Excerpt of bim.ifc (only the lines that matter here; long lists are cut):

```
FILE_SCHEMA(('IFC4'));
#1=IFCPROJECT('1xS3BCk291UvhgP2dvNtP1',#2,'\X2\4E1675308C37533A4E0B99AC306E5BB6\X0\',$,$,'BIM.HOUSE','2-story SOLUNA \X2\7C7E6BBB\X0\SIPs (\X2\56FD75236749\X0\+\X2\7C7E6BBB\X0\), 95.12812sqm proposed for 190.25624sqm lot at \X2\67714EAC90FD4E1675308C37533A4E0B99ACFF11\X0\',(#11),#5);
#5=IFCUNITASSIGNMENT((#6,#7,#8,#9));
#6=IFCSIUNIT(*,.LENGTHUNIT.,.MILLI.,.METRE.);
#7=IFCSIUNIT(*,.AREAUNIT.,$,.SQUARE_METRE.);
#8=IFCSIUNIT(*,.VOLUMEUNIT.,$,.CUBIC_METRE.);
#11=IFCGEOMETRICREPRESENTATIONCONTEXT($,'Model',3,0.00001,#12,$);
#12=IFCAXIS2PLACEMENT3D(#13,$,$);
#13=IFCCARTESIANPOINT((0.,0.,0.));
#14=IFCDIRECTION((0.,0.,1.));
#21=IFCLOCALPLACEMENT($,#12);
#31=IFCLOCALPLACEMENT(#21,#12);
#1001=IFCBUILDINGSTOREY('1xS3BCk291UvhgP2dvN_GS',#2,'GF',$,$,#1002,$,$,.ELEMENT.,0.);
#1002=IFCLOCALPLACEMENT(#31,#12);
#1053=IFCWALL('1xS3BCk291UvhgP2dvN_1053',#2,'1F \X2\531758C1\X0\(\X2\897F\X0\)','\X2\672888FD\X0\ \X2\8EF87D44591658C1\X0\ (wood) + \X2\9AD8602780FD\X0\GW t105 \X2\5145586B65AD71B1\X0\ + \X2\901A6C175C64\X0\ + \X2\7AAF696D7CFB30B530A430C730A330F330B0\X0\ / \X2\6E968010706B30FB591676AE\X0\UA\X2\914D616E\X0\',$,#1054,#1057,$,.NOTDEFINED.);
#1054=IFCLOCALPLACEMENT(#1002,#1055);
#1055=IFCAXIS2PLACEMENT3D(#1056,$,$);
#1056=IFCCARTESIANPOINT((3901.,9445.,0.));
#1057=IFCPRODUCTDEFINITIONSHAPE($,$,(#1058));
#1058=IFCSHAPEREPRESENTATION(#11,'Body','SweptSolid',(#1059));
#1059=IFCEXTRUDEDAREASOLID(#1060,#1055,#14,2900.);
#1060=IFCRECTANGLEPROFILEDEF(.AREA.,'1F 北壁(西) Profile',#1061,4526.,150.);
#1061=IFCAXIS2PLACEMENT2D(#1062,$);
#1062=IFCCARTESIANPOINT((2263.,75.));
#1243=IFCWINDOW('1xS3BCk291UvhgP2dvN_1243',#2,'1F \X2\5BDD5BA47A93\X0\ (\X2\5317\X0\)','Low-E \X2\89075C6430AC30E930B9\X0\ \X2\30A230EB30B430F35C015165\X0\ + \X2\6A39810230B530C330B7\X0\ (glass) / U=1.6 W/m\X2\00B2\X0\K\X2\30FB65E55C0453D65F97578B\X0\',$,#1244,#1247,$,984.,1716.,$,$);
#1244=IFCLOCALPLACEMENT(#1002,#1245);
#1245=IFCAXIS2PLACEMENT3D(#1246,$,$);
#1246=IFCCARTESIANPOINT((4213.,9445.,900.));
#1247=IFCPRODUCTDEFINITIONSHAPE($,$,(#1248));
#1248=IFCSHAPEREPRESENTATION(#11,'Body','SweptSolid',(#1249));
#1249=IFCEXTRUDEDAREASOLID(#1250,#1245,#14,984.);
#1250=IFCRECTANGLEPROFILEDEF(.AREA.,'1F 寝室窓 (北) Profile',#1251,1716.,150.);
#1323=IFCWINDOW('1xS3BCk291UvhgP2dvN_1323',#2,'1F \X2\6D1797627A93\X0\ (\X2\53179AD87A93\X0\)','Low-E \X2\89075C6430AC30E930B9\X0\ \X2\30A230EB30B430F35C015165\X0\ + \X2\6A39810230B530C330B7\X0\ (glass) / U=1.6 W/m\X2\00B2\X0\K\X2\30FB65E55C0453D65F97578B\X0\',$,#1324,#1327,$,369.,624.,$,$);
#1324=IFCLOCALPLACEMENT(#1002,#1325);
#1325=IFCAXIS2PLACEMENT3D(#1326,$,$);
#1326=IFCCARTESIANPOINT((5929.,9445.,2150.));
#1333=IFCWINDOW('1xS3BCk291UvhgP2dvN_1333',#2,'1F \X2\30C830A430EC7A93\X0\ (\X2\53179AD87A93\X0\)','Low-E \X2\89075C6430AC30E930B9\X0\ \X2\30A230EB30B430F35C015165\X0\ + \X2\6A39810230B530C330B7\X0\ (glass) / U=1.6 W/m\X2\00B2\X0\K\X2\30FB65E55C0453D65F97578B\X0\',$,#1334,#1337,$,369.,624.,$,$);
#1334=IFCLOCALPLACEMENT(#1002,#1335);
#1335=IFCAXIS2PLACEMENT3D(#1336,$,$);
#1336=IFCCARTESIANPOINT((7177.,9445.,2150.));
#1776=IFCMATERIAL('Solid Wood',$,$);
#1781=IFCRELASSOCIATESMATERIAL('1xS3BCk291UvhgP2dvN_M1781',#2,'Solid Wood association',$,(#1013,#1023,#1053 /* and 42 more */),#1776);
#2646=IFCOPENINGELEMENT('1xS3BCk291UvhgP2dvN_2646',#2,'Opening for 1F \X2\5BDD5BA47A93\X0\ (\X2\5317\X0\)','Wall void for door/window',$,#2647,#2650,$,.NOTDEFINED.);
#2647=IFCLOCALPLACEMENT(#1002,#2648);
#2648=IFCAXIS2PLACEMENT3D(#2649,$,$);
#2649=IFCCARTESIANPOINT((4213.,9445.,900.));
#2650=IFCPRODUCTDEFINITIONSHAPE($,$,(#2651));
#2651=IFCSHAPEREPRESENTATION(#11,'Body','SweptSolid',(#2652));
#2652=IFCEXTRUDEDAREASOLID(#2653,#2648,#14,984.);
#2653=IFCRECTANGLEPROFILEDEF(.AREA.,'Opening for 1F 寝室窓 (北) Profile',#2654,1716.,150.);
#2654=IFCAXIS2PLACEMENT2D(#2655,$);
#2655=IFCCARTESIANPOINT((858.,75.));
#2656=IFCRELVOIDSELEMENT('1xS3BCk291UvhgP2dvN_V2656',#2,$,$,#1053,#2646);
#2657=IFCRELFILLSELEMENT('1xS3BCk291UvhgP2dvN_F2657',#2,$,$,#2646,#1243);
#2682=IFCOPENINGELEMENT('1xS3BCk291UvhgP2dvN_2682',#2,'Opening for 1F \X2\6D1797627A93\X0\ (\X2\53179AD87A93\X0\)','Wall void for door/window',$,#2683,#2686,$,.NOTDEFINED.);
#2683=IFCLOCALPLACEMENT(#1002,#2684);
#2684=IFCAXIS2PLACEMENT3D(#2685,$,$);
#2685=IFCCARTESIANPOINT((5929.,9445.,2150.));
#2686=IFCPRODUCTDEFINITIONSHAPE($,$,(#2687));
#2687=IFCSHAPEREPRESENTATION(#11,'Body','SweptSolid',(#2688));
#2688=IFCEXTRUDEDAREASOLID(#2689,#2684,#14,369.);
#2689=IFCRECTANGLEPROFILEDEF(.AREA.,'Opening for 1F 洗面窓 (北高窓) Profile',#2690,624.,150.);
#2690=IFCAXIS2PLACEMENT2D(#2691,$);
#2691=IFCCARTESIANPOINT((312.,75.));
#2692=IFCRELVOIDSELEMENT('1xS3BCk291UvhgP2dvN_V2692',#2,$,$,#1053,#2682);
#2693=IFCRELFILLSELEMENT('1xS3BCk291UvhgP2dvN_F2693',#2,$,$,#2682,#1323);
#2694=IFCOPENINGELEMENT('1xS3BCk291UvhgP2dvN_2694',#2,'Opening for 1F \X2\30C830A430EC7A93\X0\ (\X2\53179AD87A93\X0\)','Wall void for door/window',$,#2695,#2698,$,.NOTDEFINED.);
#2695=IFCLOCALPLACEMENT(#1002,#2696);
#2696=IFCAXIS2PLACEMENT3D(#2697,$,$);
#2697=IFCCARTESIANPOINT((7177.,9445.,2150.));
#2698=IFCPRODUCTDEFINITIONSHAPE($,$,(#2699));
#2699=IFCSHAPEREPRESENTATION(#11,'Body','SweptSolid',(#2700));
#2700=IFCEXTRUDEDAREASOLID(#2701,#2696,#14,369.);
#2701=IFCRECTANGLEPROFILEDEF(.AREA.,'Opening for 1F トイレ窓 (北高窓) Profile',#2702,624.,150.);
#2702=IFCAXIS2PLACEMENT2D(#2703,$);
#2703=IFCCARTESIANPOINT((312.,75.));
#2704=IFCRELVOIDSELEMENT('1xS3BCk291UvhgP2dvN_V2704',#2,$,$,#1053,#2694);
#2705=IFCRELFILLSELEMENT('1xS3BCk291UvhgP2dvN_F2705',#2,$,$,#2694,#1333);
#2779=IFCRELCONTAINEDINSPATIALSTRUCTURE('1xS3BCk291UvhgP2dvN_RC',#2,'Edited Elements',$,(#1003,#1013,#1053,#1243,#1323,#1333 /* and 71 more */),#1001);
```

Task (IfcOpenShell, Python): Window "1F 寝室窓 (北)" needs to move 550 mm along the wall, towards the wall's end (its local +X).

```python
import ifcopenshell
import ifcopenshell.api.geometry
import ifcopenshell.util.placement
import ifcopenshell.util.unit

model = ifcopenshell.open("bim.ifc")
unit_scale = ifcopenshell.util.unit.calculate_unit_scale(model)

window = model.by_guid("1xS3BCk291UvhgP2dvN_1243")
opening = window.FillsVoids[0].RelatingOpeningElement
wall = opening.VoidsElements[0].RelatingBuildingElement

wall_matrix = ifcopenshell.util.placement.get_local_placement(wall.ObjectPlacement)
shift = wall_matrix[:3, 0] * 0.55 / unit_scale
before = ifcopenshell.util.placement.get_local_placement(window.ObjectPlacement)[:3, 3].copy()

# The window is not placed relative to its opening, so move both.
for product in (opening, window):
    matrix = ifcopenshell.util.placement.get_local_placement(product.ObjectPlacement)
    matrix[:3, 3] += shift
    ifcopenshell.api.geometry.edit_object_placement(model, product=product, matrix=matrix, is_si=False)

after = ifcopenshell.util.placement.get_local_placement(window.ObjectPlacement)[:3, 3]
print("window moved by", (after - before).round(3) + 0.0)

model.write("bim-out.ifc")
```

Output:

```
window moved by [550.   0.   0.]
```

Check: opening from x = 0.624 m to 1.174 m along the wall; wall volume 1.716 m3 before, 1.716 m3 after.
